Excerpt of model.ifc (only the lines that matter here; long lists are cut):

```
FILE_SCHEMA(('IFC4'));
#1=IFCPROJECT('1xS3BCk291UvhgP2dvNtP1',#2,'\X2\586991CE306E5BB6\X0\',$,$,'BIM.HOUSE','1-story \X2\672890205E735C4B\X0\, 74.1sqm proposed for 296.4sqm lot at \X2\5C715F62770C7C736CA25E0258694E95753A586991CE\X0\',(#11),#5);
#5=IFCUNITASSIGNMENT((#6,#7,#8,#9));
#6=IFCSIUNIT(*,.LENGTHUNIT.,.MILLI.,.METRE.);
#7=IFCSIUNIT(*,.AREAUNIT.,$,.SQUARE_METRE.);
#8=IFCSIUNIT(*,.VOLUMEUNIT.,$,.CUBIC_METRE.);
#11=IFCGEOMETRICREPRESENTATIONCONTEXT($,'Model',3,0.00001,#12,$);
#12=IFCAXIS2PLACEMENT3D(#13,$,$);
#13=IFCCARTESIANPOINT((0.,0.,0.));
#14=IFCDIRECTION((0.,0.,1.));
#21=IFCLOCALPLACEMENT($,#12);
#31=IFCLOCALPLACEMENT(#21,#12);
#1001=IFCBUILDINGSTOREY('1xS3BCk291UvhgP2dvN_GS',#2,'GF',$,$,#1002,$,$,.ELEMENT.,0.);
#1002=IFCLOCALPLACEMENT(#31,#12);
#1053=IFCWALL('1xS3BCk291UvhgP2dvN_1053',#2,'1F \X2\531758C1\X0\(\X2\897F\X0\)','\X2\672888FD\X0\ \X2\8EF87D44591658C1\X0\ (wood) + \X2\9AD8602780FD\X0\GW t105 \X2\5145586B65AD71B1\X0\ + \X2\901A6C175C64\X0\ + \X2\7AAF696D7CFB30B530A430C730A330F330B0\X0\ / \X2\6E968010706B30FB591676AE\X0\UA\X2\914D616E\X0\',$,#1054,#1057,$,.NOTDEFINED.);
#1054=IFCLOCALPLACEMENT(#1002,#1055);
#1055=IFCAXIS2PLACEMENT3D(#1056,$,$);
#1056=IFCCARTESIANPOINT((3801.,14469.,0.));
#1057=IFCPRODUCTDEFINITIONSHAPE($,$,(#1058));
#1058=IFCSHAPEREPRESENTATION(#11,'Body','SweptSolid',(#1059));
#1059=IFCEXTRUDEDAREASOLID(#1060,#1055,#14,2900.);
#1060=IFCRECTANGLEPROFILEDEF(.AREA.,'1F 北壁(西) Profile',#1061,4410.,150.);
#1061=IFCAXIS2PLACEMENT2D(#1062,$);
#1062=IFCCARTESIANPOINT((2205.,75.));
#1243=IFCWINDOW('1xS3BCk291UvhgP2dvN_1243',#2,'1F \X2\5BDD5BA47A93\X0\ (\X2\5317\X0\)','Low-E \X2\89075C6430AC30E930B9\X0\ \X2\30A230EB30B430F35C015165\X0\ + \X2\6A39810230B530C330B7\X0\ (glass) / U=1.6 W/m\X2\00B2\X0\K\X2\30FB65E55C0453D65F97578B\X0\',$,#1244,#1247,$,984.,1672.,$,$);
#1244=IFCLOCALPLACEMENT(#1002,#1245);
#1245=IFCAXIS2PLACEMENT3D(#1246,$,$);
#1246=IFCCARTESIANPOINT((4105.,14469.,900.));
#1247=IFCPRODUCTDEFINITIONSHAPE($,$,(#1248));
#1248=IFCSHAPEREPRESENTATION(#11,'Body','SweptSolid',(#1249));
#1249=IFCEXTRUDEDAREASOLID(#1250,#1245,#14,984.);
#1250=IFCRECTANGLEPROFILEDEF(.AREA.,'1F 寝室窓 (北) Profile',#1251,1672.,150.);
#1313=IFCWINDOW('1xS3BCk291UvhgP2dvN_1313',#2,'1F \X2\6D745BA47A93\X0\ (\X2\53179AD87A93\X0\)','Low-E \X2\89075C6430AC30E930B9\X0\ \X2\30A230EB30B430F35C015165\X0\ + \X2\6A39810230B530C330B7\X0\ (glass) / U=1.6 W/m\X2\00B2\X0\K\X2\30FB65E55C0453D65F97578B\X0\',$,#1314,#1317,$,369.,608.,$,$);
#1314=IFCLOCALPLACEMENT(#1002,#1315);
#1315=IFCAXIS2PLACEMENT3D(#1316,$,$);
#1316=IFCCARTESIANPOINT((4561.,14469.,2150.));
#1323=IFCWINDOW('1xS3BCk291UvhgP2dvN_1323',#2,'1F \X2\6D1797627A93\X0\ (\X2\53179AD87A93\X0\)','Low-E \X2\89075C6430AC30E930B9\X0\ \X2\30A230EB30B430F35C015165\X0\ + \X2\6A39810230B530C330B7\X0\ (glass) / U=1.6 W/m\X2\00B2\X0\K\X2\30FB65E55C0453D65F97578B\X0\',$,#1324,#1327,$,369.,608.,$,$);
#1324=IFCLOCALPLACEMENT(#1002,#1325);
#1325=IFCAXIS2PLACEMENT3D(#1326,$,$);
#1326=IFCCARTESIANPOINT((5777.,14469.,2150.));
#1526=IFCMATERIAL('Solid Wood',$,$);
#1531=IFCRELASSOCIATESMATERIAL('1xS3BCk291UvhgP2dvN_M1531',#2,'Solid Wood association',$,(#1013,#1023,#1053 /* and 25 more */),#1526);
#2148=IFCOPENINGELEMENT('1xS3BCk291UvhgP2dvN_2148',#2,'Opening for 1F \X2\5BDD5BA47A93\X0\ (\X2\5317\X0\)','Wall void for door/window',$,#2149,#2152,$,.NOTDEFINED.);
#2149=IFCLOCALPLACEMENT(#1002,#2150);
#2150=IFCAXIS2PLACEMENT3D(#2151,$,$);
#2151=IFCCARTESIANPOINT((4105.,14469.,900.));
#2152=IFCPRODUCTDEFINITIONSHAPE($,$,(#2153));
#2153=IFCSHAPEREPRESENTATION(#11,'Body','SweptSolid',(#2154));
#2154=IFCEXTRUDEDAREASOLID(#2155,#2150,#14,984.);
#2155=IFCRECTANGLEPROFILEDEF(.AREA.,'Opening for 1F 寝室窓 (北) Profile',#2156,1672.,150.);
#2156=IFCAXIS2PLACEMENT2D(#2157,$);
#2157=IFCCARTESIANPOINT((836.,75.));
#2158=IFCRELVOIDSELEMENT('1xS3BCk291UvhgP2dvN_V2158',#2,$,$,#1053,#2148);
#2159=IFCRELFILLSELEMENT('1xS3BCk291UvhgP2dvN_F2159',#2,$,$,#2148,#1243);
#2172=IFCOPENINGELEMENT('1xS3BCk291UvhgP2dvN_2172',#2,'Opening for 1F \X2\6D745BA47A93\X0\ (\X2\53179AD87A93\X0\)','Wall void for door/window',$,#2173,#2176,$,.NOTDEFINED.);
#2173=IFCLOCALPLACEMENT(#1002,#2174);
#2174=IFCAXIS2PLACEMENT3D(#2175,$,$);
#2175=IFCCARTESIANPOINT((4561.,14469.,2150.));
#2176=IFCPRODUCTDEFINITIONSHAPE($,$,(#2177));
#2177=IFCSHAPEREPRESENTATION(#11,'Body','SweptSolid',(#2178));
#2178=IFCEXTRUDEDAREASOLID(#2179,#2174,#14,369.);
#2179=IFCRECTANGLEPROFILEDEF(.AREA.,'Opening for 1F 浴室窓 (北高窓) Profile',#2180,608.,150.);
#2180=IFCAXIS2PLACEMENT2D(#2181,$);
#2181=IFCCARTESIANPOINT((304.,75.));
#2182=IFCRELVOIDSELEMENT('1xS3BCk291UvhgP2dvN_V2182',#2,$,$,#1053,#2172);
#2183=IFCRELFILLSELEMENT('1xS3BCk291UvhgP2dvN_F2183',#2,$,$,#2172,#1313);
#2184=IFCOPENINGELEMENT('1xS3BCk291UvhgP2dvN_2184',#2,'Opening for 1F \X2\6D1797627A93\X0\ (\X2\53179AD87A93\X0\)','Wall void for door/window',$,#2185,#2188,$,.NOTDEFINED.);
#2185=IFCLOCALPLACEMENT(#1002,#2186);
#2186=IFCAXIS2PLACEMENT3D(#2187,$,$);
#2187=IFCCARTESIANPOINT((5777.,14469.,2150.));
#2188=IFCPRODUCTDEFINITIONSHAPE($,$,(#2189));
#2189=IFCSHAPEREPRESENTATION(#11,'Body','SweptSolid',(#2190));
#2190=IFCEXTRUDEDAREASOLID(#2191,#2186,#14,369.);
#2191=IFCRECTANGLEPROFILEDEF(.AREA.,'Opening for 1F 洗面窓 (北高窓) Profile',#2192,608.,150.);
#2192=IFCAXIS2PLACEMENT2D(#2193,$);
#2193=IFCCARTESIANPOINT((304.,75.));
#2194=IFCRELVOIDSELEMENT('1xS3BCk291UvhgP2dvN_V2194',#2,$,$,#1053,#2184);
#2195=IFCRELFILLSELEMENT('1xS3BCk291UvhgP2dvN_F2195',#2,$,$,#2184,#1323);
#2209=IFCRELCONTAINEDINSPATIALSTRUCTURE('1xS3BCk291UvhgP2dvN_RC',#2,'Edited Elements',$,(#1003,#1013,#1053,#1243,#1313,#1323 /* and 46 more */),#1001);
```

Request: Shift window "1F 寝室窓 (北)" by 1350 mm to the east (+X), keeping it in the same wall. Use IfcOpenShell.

```python
import ifcopenshell
import ifcopenshell.api.geometry
import ifcopenshell.util.placement
import ifcopenshell.util.unit

model = ifcopenshell.open("model.ifc")
unit_scale = ifcopenshell.util.unit.calculate_unit_scale(model)

window = model.by_guid("1xS3BCk291UvhgP2dvN_1243")
opening = window.FillsVoids[0].RelatingOpeningElement
wall = opening.VoidsElements[0].RelatingBuildingElement

wall_matrix = ifcopenshell.util.placement.get_local_placement(wall.ObjectPlacement)
shift = wall_matrix[:3, 0] * 1.35 / unit_scale
before = ifcopenshell.util.placement.get_local_placement(window.ObjectPlacement)[:3, 3].copy()

# The window is not placed relative to its opening, so move both.
for product in (opening, window):
    matrix = ifcopenshell.util.placement.get_local_placement(product.ObjectPlacement)
    matrix[:3, 3] += shift
    ifcopenshell.api.geometry.edit_object_placement(model, product=product, matrix=matrix, is_si=False)

after = ifcopenshell.util.placement.get_local_placement(window.ObjectPlacement)[:3, 3]
print("window moved by", (after - before).round(3) + 0.0)

model.write("model_updated.ifc")
```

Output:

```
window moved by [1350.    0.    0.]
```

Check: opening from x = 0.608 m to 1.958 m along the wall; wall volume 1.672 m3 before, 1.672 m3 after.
